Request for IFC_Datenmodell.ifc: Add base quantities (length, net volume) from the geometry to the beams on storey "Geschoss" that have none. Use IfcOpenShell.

First a look at what the model holds.

```python
import ifcopenshell
import ifcopenshell.util.element
import ifcopenshell.util.unit

model = ifcopenshell.open("IFC_Datenmodell.ifc")
print(model.schema)
for unit_type in ("LENGTHUNIT", "AREAUNIT", "VOLUMEUNIT"):
    print(unit_type, ifcopenshell.util.unit.calculate_unit_scale(model, unit_type))
storey = next(s for s in model.by_type("IfcBuildingStorey") if s.Name == "Geschoss")
beams = [e for e in ifcopenshell.util.element.get_decomposition(storey) if e.is_a("IfcBeam")]
for e in sorted(beams, key=lambda e: e.id()):
    print(e.id(), e.is_a(), e.Name, list(ifcopenshell.util.element.get_psets(e, qtos_only=True)), sep=" | ")
```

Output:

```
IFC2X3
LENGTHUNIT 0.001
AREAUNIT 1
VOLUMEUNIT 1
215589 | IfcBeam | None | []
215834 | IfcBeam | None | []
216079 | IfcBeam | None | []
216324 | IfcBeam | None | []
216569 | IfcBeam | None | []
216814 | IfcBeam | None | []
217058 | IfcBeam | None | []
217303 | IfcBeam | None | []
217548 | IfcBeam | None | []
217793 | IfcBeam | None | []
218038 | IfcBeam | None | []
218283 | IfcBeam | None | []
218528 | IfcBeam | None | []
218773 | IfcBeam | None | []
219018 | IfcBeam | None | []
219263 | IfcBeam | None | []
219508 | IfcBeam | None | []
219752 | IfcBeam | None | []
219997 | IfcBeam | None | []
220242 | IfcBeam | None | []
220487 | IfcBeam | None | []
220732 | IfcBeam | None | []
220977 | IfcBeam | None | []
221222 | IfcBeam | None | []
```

```python
import ifcopenshell
import ifcopenshell.api.pset
import ifcopenshell.geom
import ifcopenshell.util.element
import ifcopenshell.util.shape
import ifcopenshell.util.unit

model = ifcopenshell.open("IFC_Datenmodell.ifc")
unit_scale = ifcopenshell.util.unit.calculate_unit_scale(model)
volume_scale = ifcopenshell.util.unit.calculate_unit_scale(model, "VOLUMEUNIT")
settings = ifcopenshell.geom.settings()

storey = next(s for s in model.by_type("IfcBuildingStorey") if s.Name == "Geschoss")
beams = [e for e in ifcopenshell.util.element.get_decomposition(storey) if e.is_a("IfcBeam")]

for e in sorted(beams, key=lambda e: e.id()):
    if ifcopenshell.util.element.get_psets(e, qtos_only=True, should_inherit=False):
        continue
    # Geometry comes back in metres, in the element's own axes.
    shape = ifcopenshell.geom.create_shape(settings, e)
    values = {
        "Length": ifcopenshell.util.shape.get_max_xyz(shape.geometry) / unit_scale,
        "NetVolume": ifcopenshell.util.shape.get_volume(shape.geometry) / volume_scale,
    }
    qto = ifcopenshell.api.pset.add_qto(model, product=e, name="BaseQuantities")
    ifcopenshell.api.pset.edit_qto(model, qto=qto, properties=values)
    print(e.id(), {k: round(v, 3) for k, v in values.items()})

model.write("IFC_Datenmodell_rev.ifc")
```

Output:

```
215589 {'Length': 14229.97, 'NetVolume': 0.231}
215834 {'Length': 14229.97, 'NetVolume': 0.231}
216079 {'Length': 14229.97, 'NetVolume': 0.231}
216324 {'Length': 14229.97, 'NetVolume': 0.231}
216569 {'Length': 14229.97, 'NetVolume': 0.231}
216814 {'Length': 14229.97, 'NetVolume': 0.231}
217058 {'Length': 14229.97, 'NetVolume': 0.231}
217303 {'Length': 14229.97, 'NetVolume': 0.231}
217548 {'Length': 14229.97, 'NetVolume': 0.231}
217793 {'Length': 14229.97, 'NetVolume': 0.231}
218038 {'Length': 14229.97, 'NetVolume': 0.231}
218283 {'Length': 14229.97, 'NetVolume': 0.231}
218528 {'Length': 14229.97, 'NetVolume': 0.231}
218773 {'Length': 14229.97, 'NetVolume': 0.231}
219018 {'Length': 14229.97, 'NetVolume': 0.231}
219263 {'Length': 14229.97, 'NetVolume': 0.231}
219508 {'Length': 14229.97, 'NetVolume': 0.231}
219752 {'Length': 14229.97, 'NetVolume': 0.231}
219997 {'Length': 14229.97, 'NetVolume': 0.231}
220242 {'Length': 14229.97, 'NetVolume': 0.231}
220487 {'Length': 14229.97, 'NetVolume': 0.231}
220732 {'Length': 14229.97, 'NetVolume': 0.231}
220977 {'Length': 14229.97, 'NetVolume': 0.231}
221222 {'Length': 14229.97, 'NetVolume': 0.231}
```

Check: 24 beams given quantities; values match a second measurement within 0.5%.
